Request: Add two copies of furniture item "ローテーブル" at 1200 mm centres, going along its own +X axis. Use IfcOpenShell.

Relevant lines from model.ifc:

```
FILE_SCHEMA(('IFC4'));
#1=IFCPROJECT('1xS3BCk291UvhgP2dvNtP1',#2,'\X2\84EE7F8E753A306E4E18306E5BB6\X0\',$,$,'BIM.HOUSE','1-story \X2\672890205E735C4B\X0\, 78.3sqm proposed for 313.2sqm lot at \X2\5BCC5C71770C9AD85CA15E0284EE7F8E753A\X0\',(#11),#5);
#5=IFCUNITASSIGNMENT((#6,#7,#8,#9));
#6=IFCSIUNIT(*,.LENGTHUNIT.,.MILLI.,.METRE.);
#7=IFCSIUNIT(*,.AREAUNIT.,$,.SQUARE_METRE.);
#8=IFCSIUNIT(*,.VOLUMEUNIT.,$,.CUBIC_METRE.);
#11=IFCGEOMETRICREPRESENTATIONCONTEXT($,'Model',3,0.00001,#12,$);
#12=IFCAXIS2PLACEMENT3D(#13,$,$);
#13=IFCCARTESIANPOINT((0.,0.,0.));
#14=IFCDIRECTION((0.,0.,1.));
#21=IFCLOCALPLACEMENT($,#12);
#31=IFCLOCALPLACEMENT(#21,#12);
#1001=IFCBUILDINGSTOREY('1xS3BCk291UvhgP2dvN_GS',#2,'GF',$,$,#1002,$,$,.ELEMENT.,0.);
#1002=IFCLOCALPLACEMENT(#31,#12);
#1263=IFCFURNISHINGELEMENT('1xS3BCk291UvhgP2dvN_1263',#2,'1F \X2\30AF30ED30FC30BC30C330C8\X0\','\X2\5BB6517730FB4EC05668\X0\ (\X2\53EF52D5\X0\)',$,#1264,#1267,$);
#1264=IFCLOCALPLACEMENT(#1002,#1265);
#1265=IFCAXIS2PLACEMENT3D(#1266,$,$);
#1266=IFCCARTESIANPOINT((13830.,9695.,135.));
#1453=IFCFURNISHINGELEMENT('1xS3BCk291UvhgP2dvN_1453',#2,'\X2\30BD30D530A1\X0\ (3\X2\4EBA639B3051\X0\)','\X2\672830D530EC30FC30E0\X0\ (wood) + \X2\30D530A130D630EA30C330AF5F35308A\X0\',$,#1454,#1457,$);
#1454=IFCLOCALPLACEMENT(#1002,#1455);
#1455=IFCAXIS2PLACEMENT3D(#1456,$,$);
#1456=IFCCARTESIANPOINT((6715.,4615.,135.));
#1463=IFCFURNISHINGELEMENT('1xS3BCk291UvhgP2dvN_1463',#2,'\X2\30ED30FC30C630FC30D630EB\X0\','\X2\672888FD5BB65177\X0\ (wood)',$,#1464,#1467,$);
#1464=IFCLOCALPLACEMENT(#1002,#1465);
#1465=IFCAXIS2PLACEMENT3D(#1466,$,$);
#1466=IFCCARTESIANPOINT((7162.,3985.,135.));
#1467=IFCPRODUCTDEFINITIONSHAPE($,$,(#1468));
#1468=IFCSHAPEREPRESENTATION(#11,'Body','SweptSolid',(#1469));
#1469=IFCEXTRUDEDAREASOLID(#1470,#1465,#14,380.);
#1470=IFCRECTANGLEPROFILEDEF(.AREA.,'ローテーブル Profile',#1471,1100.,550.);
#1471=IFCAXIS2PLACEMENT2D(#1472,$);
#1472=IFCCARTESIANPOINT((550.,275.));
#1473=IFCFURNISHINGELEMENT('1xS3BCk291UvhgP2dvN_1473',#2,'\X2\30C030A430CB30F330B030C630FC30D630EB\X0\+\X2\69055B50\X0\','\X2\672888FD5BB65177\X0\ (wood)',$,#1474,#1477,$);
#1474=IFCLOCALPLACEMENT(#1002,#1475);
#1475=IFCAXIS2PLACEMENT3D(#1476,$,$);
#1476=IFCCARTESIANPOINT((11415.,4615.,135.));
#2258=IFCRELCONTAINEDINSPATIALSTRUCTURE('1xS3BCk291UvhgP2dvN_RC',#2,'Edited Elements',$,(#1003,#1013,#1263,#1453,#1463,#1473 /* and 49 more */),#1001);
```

```python
import ifcopenshell
import ifcopenshell.api.geometry
import ifcopenshell.api.root
import ifcopenshell.util.element
import ifcopenshell.util.placement
import ifcopenshell.util.unit

model = ifcopenshell.open("model.ifc")
unit_scale = ifcopenshell.util.unit.calculate_unit_scale(model)


def reuse_history(source, copy):
    """copy_class also copies each property set's owner history, people and application; keep the originals."""
    for rel in copy.IsDefinedBy:
        if rel.is_a("IfcRelDefinesByProperties") and (history := rel.RelatingPropertyDefinition.OwnerHistory):
            rel.RelatingPropertyDefinition.OwnerHistory = source.OwnerHistory
            ifcopenshell.util.element.remove_deep2(model, history)


source = model.by_guid("1xS3BCk291UvhgP2dvN_1463")
base = ifcopenshell.util.placement.get_local_placement(source.ObjectPlacement)
step = base[:3, 0] * 1.2 / unit_scale

for i in range(1, 3):
    copy = ifcopenshell.api.root.copy_class(model, product=source)
    copy.Representation = ifcopenshell.util.element.copy_deep(
        model, source.Representation, exclude=["IfcGeometricRepresentationContext", "IfcRepresentationMap"]
    )
    reuse_history(source, copy)
    matrix = base.copy()
    matrix[:3, 3] += i * step
    print("added at", matrix[:3, 3].round(3) + 0.0)
    ifcopenshell.api.geometry.edit_object_placement(model, product=copy, matrix=matrix, is_si=False)

model.write("model_v2.ifc")
```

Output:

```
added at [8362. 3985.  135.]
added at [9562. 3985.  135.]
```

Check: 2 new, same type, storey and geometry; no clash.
